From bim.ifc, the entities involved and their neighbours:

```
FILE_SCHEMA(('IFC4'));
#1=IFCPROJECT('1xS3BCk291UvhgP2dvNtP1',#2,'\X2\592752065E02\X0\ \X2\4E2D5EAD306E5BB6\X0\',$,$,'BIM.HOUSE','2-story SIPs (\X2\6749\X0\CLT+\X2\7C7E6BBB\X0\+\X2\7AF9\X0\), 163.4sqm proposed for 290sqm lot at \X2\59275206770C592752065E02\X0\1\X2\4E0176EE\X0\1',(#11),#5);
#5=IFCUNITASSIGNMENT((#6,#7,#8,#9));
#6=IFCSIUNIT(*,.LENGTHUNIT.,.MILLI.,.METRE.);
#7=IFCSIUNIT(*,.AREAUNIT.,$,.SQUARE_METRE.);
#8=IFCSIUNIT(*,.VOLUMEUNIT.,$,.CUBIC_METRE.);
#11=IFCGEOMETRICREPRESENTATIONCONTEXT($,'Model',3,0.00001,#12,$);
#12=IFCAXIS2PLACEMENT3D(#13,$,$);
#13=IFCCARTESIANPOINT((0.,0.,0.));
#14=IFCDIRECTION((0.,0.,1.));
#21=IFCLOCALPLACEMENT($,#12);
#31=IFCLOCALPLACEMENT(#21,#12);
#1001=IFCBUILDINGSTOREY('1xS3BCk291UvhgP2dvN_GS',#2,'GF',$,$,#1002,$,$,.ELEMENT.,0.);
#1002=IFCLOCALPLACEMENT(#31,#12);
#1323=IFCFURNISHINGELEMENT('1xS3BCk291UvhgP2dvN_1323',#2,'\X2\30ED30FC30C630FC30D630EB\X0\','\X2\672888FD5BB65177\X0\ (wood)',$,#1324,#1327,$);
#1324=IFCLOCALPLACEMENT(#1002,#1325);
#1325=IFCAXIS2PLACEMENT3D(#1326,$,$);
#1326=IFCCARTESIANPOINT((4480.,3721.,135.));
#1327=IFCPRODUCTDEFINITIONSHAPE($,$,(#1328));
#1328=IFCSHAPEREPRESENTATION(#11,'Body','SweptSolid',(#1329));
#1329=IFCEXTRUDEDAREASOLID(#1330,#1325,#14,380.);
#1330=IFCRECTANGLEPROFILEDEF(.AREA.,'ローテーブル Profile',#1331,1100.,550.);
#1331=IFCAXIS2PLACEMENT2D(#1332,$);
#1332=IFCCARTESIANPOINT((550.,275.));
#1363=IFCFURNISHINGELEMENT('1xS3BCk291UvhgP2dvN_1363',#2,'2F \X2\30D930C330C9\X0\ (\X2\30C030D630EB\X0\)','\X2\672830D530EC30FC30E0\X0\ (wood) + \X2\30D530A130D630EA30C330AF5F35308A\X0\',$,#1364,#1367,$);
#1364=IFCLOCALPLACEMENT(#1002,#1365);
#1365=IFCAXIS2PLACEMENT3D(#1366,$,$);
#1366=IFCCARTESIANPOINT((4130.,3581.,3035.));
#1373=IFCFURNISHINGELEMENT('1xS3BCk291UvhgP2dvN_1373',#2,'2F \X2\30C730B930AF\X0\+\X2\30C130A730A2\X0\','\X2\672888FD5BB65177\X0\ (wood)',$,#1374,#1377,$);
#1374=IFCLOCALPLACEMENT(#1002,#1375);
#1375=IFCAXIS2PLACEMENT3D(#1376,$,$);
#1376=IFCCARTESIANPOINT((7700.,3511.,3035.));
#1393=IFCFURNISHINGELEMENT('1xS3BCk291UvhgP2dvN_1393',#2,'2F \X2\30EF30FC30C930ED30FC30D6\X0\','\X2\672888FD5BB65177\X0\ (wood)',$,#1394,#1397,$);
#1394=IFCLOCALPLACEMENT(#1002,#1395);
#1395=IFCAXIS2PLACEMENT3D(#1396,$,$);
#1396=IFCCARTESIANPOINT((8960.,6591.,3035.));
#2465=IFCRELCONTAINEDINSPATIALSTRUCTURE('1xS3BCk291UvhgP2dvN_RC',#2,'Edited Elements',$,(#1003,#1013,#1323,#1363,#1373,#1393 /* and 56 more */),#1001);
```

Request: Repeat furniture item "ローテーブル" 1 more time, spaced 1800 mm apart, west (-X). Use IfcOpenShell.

```python
import numpy as np
import ifcopenshell
import ifcopenshell.api.geometry
import ifcopenshell.api.root
import ifcopenshell.util.element
import ifcopenshell.util.placement

model = ifcopenshell.open("bim.ifc")


def reuse_history(source, copy):
    """copy_class also copies each property set's owner history, people and application; keep the originals."""
    for rel in copy.IsDefinedBy:
        if rel.is_a("IfcRelDefinesByProperties") and (history := rel.RelatingPropertyDefinition.OwnerHistory):
            rel.RelatingPropertyDefinition.OwnerHistory = source.OwnerHistory
            ifcopenshell.util.element.remove_deep2(model, history)


source = model.by_guid("1xS3BCk291UvhgP2dvN_1323")
base = ifcopenshell.util.placement.get_local_placement(source.ObjectPlacement)
step = np.array([-1.0, 0.0, 0.0]) * 1800.0

for i in range(1, 2):
    copy = ifcopenshell.api.root.copy_class(model, product=source)
    copy.Representation = ifcopenshell.util.element.copy_deep(
        model, source.Representation, exclude=["IfcGeometricRepresentationContext", "IfcRepresentationMap"]
    )
    reuse_history(source, copy)
    matrix = base.copy()
    matrix[:3, 3] += i * step
    print("added at", matrix[:3, 3].round(3) + 0.0)
    ifcopenshell.api.geometry.edit_object_placement(model, product=copy, matrix=matrix, is_si=False)

model.write("bim_v2.ifc")
```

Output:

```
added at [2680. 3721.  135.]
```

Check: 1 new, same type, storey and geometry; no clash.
